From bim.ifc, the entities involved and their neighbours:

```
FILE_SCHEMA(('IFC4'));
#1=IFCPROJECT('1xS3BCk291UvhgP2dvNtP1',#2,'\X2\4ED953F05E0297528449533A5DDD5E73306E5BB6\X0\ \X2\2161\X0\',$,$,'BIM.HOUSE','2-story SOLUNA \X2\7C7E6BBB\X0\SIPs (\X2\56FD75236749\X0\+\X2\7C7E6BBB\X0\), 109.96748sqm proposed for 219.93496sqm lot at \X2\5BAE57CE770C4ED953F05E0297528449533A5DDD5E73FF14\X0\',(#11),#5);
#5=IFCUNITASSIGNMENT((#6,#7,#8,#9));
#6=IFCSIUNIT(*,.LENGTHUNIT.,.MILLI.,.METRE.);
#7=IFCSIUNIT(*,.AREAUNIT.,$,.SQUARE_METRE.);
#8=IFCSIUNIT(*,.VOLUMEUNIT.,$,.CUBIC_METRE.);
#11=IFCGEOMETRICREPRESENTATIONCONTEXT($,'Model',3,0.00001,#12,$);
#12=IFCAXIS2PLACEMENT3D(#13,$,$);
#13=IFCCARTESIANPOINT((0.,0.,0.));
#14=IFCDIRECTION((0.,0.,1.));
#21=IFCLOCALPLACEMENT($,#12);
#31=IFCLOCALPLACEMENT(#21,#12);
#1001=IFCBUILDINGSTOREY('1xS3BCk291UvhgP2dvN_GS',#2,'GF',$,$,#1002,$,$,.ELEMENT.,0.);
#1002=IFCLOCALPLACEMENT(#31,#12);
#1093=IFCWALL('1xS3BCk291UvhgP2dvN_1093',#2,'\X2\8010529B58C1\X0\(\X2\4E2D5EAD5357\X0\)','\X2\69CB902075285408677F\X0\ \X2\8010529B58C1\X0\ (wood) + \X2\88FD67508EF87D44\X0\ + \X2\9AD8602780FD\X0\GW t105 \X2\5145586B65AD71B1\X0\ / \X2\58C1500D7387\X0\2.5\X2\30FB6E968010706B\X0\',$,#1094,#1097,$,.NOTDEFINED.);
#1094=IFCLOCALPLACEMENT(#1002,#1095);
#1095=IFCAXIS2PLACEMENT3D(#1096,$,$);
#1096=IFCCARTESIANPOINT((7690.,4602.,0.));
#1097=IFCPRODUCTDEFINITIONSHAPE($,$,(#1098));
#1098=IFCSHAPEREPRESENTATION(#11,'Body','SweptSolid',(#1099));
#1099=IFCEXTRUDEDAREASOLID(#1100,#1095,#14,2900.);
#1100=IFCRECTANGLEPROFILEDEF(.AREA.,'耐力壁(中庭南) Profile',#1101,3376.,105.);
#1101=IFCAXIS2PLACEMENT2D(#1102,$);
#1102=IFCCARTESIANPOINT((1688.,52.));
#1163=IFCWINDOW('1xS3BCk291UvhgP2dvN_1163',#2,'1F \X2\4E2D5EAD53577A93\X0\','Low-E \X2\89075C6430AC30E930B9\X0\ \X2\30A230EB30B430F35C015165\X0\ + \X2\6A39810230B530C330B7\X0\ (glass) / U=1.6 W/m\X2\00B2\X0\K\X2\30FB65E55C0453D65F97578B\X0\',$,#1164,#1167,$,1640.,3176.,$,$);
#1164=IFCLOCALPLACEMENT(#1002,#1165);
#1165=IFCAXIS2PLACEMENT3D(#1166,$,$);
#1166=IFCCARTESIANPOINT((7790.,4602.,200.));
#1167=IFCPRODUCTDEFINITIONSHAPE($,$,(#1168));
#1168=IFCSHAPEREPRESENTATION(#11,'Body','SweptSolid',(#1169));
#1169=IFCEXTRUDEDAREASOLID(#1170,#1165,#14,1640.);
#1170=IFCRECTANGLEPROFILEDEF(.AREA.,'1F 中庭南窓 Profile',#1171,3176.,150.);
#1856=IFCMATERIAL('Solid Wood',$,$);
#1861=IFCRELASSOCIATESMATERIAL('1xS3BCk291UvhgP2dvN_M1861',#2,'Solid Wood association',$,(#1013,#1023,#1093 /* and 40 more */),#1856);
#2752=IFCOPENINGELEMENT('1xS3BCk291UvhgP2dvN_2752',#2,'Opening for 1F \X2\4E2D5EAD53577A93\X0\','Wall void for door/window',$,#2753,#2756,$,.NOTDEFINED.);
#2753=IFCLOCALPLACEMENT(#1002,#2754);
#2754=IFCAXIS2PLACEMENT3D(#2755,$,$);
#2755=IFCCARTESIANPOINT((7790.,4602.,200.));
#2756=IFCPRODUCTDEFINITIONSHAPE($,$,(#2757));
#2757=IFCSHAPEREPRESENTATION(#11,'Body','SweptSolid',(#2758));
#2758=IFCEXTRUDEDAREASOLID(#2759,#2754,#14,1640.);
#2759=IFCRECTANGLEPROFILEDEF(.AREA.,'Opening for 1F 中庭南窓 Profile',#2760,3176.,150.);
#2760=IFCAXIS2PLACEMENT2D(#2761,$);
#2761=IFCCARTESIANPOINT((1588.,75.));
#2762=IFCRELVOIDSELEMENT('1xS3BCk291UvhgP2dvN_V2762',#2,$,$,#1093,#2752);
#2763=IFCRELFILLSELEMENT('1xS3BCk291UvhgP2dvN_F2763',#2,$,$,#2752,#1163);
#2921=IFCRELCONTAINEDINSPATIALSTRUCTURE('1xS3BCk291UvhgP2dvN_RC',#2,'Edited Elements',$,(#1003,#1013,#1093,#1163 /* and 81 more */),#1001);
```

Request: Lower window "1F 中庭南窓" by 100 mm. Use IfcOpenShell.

```python
import numpy as np
import ifcopenshell
import ifcopenshell.api.geometry
import ifcopenshell.util.placement
import ifcopenshell.util.unit

model = ifcopenshell.open("bim.ifc")
unit_scale = ifcopenshell.util.unit.calculate_unit_scale(model)

window = model.by_guid("1xS3BCk291UvhgP2dvN_1163")
opening = window.FillsVoids[0].RelatingOpeningElement
dz = -100.0

shift = np.array([0.0, 0.0, dz])
# The window is not placed relative to its opening, so move both.
for product in (opening, window):
    matrix = ifcopenshell.util.placement.get_local_placement(product.ObjectPlacement)
    matrix[:3, 3] += shift
    ifcopenshell.api.geometry.edit_object_placement(model, product=product, matrix=matrix, is_si=False)

print(f"moved by {dz * unit_scale:+.3f} m")

model.write("bim_updated.ifc")
```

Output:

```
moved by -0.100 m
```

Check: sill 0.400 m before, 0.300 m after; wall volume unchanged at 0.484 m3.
